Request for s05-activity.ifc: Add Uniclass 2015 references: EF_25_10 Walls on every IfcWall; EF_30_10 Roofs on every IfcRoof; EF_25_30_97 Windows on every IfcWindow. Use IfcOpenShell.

First a look at what the model holds.

```python
import ifcopenshell

model = ifcopenshell.open("s05-activity.ifc")
print(model.schema)
print("classifications:", [c.Name for c in model.by_type("IfcClassification")])
for ifc_class in ("IfcDoor", "IfcRoof", "IfcStair", "IfcWall", "IfcWindow"):
    print(ifc_class, len(model.by_type(ifc_class)))
```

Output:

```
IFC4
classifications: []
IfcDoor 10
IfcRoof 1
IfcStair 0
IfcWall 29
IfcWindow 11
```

```python
import ifcopenshell
import ifcopenshell.api.classification

model = ifcopenshell.open("s05-activity.ifc")

system = ifcopenshell.api.classification.add_classification(model, classification="Uniclass 2015")

codes = {
    "IfcWall": ("EF_25_10", "Walls"),
    "IfcRoof": ("EF_30_10", "Roofs"),
    "IfcWindow": ("EF_25_30_97", "Windows"),
}
for ifc_class, (code, name) in codes.items():
    products = model.by_type(ifc_class)
    ifcopenshell.api.classification.add_reference(
        model, products=products, classification=system, identification=code, name=name
    )
    print(code, len(products))

model.write("s05-activity_updated.ifc")
```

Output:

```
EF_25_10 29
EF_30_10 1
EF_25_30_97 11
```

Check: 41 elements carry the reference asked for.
